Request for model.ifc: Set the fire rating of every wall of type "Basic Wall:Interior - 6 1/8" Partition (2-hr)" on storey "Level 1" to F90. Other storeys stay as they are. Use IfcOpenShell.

First a look at what the model holds.

```python
import ifcopenshell
import ifcopenshell.util.element

model = ifcopenshell.open("model.ifc")
print(model.schema)
storey = next(s for s in model.by_type("IfcBuildingStorey") if s.Name == "Level 1")
walls = [e for e in ifcopenshell.util.element.get_decomposition(storey) if e.is_a("IfcWall")]
seen = {}
for e in walls:
    element_type = ifcopenshell.util.element.get_type(e)
    key = (element_type.Name if element_type != e and element_type else None, ifcopenshell.util.element.get_pset(e, "Pset_WallCommon", "FireRating"))
    seen[key] = seen.get(key, 0) + 1
for (name, value), count in sorted(seen.items(), key=str):
    print(count, "x", name, "|", value)
```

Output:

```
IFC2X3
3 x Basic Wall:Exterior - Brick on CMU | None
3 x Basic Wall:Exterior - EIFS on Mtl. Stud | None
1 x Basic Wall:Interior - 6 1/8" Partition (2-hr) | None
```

```python
import ifcopenshell
import ifcopenshell.api.pset
import ifcopenshell.util.element

model = ifcopenshell.open("model.ifc")

storey = next(s for s in model.by_type("IfcBuildingStorey") if s.Name == "Level 1")
walls = [e for e in ifcopenshell.util.element.get_decomposition(storey) if e.is_a("IfcWall")]

count = 0
for e in walls:
    element_type = ifcopenshell.util.element.get_type(e)
    if element_type in (None, e) or element_type.Name != 'Basic Wall:Interior - 6 1/8" Partition (2-hr)':
        continue
    # add_pset returns the element's existing set when there is one.
    pset = ifcopenshell.api.pset.add_pset(model, product=e, name="Pset_WallCommon")
    ifcopenshell.api.pset.edit_pset(model, pset=pset, properties={"FireRating": "F90"})
    count += 1

print(count, "walls updated")

model.write("model_edited.ifc")
```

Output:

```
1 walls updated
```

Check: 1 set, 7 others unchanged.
